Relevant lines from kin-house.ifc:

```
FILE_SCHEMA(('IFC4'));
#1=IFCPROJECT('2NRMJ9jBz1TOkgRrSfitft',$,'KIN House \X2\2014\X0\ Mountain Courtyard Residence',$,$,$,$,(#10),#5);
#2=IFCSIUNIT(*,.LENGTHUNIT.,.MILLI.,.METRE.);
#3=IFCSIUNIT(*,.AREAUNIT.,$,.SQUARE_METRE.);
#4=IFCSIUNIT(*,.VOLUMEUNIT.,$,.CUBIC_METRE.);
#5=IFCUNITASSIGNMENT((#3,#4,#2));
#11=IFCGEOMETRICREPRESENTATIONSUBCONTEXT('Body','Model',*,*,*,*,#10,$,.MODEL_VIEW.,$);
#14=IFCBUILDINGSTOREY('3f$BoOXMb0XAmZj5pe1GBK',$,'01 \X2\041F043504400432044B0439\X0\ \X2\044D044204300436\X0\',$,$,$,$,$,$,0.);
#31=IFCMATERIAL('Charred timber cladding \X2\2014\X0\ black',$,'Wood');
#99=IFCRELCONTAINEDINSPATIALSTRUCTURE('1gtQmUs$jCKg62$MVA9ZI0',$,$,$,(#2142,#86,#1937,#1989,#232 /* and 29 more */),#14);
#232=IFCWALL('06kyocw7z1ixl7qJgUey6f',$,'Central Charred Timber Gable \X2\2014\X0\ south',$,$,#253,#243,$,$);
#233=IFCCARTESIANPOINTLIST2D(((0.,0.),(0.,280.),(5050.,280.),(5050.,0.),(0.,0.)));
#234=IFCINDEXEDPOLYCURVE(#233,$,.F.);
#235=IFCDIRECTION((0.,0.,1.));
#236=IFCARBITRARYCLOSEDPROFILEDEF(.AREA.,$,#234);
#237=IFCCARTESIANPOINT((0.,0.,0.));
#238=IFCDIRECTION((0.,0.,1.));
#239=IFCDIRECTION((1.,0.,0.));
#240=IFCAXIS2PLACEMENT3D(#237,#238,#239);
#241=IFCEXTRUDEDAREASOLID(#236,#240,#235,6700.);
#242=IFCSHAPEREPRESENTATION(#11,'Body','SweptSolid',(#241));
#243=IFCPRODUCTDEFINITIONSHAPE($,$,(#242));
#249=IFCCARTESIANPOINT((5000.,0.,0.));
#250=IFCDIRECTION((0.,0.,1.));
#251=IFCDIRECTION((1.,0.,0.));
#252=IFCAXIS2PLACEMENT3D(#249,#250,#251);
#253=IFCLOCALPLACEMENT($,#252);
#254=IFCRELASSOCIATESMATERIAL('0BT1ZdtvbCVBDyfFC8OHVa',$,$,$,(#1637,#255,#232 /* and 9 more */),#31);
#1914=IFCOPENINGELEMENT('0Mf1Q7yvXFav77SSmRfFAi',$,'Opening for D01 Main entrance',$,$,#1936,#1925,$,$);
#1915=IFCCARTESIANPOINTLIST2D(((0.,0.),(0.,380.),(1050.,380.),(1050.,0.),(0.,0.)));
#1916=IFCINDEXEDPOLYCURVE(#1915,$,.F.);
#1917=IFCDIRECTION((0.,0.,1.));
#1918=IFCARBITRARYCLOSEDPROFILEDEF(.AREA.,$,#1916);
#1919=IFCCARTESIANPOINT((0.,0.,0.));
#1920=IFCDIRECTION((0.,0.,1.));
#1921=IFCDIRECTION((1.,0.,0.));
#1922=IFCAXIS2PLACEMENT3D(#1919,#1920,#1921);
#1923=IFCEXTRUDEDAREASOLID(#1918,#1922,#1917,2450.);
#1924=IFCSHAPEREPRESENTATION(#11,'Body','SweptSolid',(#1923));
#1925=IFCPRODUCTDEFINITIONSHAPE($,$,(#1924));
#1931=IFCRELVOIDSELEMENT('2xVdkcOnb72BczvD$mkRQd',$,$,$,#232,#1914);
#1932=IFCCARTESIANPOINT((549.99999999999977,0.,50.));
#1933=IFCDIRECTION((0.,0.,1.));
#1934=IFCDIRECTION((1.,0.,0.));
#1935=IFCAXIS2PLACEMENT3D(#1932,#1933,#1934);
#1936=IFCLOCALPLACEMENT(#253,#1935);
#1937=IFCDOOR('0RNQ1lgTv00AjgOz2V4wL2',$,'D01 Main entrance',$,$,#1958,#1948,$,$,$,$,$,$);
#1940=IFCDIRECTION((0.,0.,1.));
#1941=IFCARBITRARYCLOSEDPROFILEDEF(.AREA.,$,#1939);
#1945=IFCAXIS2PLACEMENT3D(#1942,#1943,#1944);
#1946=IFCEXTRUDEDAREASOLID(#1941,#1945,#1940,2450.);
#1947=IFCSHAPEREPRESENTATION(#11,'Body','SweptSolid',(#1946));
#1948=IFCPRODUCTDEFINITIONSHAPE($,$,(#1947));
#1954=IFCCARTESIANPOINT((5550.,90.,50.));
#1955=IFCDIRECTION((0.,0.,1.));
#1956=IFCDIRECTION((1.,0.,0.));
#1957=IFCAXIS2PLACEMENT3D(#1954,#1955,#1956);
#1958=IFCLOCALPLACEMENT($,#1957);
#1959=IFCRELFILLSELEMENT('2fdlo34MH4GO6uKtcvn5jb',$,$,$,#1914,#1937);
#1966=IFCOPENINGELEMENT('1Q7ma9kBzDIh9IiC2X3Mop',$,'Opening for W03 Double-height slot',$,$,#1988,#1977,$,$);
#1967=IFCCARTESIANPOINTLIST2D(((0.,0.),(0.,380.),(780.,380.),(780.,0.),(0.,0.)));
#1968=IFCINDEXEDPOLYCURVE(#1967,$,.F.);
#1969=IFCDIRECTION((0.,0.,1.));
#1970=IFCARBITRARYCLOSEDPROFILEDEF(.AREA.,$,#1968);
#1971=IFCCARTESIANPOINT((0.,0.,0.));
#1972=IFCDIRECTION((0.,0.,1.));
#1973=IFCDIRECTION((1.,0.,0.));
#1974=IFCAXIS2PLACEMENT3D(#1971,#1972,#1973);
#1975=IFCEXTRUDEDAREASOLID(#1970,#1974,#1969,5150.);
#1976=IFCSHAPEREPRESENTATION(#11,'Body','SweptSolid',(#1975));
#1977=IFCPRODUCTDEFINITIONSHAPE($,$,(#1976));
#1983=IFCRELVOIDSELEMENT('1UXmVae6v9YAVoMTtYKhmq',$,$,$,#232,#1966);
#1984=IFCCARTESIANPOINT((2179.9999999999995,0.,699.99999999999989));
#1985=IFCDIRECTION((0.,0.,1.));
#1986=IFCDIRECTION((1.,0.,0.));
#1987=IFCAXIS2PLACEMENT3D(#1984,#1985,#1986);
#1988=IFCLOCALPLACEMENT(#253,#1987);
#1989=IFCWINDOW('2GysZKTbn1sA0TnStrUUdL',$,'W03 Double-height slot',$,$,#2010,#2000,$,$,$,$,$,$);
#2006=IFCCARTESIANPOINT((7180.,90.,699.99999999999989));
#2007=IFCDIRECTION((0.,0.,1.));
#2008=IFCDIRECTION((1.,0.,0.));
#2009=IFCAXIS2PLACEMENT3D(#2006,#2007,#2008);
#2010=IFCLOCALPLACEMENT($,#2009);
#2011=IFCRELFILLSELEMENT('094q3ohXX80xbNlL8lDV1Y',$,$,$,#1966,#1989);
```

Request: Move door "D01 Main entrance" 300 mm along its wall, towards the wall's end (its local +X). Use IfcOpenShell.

```python
import ifcopenshell
import ifcopenshell.api.geometry
import ifcopenshell.util.placement

model = ifcopenshell.open("kin-house.ifc")

door = model.by_guid("0RNQ1lgTv00AjgOz2V4wL2")
opening = door.FillsVoids[0].RelatingOpeningElement
wall = opening.VoidsElements[0].RelatingBuildingElement

wall_matrix = ifcopenshell.util.placement.get_local_placement(wall.ObjectPlacement)
shift = wall_matrix[:3, 0] * 300.0
before = ifcopenshell.util.placement.get_local_placement(door.ObjectPlacement)[:3, 3].copy()

# The door is not placed relative to its opening, so move both.
for product in (opening, door):
    matrix = ifcopenshell.util.placement.get_local_placement(product.ObjectPlacement)
    matrix[:3, 3] += shift
    ifcopenshell.api.geometry.edit_object_placement(model, product=product, matrix=matrix, is_si=False)

after = ifcopenshell.util.placement.get_local_placement(door.ObjectPlacement)[:3, 3]
print("door moved by", (after - before).round(3) + 0.0)

model.write("kin-house_edited.ifc")
```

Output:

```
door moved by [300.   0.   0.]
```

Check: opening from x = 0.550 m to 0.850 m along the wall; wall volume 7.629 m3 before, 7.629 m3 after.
